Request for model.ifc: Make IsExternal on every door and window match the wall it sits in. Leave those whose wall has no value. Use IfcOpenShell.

First a look at what the model holds.

```python
import ifcopenshell
import ifcopenshell.util.element

model = ifcopenshell.open("model.ifc")
print(model.schema)
seen = {}
for e in model.by_type("IfcDoor") + model.by_type("IfcWindow"):
    if not e.FillsVoids:
        continue
    host = e.FillsVoids[0].RelatingOpeningElement.VoidsElements[0].RelatingBuildingElement
    own = ifcopenshell.util.element.get_pset(e, f"Pset_{e.is_a()[3:].removesuffix('StandardCase')}Common", "IsExternal")
    wall = ifcopenshell.util.element.get_pset(host, "Pset_WallCommon", "IsExternal")
    seen[e.is_a(), own, wall] = seen.get((e.is_a(), own, wall), 0) + 1
for (cls, own, wall), count in sorted(seen.items(), key=str):
    print(count, cls, "IsExternal:", own, "| host wall:", wall)
```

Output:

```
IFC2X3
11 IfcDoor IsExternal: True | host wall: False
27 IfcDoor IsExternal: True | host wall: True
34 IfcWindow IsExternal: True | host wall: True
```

```python
import ifcopenshell
import ifcopenshell.api.pset
import ifcopenshell.util.element

model = ifcopenshell.open("model.ifc")

count = 0
for ifc_class, pset_name in (("IfcDoor", "Pset_DoorCommon"), ("IfcWindow", "Pset_WindowCommon")):
    for e in model.by_type(ifc_class):
        if not e.FillsVoids:
            continue
        host = e.FillsVoids[0].RelatingOpeningElement.VoidsElements[0].RelatingBuildingElement
        external = ifcopenshell.util.element.get_pset(host, "Pset_WallCommon", "IsExternal")
        if external is None or ifcopenshell.util.element.get_pset(e, pset_name, "IsExternal") == external:
            continue
        pset = ifcopenshell.api.pset.add_pset(model, product=e, name=pset_name)
        ifcopenshell.api.pset.edit_pset(model, pset=pset, properties={"IsExternal": external})
        count += 1

print(count, "updated")

model.write("model_rev.ifc")
```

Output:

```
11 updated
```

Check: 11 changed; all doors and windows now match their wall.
